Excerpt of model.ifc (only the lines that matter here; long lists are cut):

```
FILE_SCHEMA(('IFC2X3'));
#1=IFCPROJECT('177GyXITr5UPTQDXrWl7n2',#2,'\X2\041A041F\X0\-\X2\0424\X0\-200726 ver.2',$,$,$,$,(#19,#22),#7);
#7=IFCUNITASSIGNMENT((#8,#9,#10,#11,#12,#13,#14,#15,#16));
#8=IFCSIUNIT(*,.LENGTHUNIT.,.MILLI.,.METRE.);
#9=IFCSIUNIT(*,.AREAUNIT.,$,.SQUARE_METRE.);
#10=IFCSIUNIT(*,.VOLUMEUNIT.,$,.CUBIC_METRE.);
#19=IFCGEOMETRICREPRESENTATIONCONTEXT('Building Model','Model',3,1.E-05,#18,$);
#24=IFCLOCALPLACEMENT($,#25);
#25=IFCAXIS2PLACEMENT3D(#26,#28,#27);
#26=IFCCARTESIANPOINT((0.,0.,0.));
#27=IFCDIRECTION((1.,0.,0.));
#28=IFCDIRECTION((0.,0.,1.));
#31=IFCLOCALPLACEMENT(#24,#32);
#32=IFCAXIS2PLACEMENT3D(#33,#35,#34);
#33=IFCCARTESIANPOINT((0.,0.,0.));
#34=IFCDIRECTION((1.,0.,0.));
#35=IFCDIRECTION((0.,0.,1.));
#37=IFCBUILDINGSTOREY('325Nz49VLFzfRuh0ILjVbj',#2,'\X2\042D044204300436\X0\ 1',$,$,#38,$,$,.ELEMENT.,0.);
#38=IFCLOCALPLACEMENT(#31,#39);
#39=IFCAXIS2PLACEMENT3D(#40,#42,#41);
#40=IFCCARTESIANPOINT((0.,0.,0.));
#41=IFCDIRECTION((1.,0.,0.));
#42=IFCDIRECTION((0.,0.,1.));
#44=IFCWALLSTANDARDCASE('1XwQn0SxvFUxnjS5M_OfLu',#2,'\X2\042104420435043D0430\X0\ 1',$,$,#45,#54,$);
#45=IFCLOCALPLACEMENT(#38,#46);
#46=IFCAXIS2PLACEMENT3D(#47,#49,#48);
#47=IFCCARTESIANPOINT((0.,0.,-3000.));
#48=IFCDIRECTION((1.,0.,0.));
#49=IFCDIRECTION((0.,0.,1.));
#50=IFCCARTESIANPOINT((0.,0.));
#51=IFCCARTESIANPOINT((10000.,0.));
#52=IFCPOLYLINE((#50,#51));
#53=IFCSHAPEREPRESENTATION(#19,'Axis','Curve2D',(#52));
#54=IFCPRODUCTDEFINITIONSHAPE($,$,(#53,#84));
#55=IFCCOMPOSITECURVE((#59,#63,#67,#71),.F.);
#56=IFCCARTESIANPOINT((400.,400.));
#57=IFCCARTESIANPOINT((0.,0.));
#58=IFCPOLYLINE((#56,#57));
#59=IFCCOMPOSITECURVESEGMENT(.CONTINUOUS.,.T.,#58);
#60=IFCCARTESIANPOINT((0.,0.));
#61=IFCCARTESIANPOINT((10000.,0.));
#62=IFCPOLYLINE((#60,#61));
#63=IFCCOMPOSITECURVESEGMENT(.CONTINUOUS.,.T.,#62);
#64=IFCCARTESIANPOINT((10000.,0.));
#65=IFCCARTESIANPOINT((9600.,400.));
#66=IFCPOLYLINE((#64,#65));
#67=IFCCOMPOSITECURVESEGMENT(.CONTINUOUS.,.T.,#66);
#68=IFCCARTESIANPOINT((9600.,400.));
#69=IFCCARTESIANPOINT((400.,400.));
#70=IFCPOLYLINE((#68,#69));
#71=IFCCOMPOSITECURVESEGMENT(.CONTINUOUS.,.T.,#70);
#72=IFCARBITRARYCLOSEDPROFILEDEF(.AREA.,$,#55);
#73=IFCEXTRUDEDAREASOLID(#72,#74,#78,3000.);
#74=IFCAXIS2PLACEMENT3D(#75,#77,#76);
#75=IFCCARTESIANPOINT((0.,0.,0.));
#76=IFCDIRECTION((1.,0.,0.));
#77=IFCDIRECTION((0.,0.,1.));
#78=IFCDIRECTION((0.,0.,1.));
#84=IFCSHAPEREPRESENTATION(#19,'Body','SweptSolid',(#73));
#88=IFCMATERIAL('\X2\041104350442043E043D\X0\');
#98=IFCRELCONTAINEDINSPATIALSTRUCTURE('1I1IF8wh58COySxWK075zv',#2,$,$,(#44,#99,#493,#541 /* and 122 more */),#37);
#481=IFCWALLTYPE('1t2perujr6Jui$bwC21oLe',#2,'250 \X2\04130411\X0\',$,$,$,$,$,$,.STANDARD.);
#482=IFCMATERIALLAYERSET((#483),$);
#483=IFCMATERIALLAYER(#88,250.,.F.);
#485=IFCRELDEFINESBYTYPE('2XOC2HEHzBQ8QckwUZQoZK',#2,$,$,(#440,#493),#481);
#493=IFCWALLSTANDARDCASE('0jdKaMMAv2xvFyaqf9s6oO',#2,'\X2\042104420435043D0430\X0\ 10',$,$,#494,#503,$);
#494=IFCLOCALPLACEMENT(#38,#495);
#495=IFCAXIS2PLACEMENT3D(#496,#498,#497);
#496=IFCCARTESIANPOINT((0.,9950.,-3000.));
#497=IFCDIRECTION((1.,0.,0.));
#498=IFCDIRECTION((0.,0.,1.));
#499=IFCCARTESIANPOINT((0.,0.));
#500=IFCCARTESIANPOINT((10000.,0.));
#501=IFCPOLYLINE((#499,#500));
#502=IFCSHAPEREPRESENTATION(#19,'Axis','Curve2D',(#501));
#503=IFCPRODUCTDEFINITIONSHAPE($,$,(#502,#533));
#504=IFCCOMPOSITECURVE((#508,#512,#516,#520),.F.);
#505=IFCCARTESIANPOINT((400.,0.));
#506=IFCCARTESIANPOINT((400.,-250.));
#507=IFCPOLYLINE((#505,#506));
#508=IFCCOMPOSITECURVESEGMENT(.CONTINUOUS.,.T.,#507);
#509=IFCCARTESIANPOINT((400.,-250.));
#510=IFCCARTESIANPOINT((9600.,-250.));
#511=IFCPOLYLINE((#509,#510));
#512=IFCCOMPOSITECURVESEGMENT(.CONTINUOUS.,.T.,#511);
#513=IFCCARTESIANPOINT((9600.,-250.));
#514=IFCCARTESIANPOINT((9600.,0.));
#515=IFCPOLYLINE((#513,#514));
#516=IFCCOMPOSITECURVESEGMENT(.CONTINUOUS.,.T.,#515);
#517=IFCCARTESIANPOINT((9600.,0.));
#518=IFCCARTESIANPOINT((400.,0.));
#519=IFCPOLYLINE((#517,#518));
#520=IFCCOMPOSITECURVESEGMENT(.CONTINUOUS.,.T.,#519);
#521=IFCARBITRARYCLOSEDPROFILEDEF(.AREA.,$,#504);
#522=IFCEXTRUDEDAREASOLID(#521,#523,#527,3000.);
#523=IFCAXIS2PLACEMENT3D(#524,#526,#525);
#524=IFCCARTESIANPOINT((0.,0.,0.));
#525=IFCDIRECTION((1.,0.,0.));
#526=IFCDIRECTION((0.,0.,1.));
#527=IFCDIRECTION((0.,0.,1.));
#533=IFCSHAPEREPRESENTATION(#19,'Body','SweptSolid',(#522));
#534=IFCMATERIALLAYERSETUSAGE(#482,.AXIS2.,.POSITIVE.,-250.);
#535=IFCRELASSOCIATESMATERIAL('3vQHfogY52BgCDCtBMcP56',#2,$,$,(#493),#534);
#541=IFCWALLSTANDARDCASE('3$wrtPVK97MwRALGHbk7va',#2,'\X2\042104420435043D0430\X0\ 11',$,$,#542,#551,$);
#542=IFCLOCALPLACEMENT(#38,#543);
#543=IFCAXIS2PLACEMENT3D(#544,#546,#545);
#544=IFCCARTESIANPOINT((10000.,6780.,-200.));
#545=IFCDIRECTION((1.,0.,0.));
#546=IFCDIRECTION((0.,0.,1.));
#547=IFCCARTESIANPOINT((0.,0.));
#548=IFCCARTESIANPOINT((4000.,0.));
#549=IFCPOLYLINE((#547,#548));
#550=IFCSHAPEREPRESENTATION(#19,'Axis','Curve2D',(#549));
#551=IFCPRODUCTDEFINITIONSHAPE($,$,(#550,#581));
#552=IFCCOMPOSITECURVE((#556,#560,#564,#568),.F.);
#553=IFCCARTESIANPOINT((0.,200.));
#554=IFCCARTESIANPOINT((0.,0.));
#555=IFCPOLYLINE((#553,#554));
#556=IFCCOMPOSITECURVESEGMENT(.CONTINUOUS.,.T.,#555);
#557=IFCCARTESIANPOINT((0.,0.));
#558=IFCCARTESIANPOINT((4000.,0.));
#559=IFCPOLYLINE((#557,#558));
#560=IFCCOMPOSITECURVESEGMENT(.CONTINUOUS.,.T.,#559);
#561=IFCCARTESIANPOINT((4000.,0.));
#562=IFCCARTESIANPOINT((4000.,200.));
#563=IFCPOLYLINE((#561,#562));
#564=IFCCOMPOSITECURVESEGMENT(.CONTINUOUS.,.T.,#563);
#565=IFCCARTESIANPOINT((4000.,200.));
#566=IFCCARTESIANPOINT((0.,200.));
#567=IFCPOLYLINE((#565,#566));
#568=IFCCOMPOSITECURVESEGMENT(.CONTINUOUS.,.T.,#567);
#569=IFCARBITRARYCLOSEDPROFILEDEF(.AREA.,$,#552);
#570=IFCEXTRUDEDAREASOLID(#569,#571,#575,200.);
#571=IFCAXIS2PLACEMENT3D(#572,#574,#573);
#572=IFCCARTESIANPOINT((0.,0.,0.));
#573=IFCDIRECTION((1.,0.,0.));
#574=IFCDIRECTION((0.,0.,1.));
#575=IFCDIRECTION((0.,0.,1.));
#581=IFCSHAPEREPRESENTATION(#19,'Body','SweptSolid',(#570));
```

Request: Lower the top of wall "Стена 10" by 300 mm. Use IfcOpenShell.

```python
import ifcopenshell
import ifcopenshell.geom
import ifcopenshell.util.shape
import ifcopenshell.util.unit

model = ifcopenshell.open("model.ifc")
unit_scale = ifcopenshell.util.unit.calculate_unit_scale(model)
settings = ifcopenshell.geom.settings()


def volume(element):
    """Net volume in cubic metres, openings subtracted."""
    shape = ifcopenshell.geom.create_shape(settings, element)
    return ifcopenshell.util.shape.get_volume(shape.geometry)


wall = model.by_guid("0jdKaMMAv2xvFyaqf9s6oO")
before = volume(wall)

body = next(r for r in wall.Representation.Representations if r.RepresentationIdentifier == "Body")
solid = body.Items[0]
old_height = solid.Depth
solid.Depth -= 0.3 / unit_scale
after = volume(wall)

print(f"height {old_height:g} -> {solid.Depth:g}, volume {before:.3f} -> {after:.3f} m3")

model.write("model_edited.ifc")
```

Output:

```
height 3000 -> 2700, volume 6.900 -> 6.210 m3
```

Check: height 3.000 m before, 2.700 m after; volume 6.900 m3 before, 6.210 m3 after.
